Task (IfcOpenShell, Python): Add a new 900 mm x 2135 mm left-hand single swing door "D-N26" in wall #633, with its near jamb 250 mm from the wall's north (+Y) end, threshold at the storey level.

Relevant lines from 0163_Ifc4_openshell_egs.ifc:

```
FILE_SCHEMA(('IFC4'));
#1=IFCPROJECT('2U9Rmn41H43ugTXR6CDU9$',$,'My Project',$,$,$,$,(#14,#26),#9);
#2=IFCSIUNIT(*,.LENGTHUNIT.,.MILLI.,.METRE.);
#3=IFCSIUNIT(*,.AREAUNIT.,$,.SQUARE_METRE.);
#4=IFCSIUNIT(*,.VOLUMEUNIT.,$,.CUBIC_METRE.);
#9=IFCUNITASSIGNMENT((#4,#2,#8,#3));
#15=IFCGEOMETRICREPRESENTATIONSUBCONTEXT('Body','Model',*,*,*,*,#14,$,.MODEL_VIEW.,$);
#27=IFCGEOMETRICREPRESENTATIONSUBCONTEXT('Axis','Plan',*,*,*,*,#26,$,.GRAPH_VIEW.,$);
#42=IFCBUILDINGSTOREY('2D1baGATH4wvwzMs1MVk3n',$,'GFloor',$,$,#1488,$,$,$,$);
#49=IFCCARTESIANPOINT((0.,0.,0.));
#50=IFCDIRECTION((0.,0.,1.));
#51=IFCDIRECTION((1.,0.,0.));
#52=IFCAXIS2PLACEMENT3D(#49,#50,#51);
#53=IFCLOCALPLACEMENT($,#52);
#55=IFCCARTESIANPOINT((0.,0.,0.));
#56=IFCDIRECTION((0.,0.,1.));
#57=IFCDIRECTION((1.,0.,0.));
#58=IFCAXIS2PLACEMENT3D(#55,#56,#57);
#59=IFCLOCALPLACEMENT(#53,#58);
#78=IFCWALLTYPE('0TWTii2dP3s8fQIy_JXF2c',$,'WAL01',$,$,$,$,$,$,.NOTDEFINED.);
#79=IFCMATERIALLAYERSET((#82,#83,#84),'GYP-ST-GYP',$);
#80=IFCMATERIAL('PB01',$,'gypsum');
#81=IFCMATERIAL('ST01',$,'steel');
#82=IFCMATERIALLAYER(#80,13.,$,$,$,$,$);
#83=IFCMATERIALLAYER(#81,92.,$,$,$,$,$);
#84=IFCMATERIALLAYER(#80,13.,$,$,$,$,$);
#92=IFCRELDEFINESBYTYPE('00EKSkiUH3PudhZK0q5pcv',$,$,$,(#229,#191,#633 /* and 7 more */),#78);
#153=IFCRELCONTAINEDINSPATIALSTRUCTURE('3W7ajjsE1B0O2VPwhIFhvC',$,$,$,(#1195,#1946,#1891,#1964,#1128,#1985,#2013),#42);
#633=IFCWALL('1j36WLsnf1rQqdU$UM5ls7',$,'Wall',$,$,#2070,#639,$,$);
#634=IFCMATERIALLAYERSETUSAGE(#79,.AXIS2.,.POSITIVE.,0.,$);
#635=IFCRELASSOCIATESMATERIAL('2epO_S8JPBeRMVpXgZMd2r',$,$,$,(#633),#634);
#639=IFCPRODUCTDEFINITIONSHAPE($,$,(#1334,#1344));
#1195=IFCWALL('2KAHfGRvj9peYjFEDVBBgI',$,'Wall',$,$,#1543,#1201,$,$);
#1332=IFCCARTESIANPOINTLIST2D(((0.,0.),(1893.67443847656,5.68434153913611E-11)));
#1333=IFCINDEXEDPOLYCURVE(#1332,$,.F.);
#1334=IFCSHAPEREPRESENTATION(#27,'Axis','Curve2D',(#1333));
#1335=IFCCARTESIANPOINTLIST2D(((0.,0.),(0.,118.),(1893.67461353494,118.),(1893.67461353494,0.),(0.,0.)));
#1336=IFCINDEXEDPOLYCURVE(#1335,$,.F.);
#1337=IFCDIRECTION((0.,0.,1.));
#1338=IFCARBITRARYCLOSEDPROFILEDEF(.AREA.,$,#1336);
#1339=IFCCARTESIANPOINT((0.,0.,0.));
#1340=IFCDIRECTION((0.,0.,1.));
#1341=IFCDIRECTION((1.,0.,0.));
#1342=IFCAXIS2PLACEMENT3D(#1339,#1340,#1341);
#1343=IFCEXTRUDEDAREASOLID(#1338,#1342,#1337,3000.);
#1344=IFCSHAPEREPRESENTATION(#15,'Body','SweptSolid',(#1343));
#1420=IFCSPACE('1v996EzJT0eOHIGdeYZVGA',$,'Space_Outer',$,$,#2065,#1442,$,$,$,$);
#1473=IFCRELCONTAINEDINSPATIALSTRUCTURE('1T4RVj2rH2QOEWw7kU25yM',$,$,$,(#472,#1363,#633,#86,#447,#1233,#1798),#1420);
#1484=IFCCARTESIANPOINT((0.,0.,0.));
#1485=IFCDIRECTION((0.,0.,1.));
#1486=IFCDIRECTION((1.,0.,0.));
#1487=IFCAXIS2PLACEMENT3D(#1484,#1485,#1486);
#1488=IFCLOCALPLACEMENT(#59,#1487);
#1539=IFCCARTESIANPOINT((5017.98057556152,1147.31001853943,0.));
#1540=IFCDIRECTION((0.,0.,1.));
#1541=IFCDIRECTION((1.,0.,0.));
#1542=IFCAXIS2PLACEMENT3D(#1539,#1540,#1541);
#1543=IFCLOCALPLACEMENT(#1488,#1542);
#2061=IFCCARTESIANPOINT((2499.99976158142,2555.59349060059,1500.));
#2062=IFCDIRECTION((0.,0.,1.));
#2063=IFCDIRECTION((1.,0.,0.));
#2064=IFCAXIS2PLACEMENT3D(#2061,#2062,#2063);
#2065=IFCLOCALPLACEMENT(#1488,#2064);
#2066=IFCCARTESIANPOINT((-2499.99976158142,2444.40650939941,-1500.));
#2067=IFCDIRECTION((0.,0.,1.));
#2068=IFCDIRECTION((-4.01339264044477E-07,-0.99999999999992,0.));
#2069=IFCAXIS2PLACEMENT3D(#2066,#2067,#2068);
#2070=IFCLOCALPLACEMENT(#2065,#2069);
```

```python
import numpy as np
import ifcopenshell
import ifcopenshell.api.feature
import ifcopenshell.api.geometry
import ifcopenshell.api.root
import ifcopenshell.api.spatial
import ifcopenshell.geom
import ifcopenshell.util.element
import ifcopenshell.util.placement
import ifcopenshell.util.representation
import ifcopenshell.util.shape
import ifcopenshell.util.unit

model = ifcopenshell.open("0163_Ifc4_openshell_egs.ifc")
unit_scale = ifcopenshell.util.unit.calculate_unit_scale(model)
settings = ifcopenshell.geom.settings()


def volume(element):
    """Net volume in cubic metres, openings subtracted."""
    shape = ifcopenshell.geom.create_shape(settings, element)
    return ifcopenshell.util.shape.get_volume(shape.geometry)


wall = model.by_guid("1j36WLsnf1rQqdU$UM5ls7")
storey = ifcopenshell.util.element.get_container(wall, ifc_class="IfcBuildingStorey")
context = ifcopenshell.util.representation.get_context(model, "Model", "Body", "MODEL_VIEW")
before = volume(wall)

width, height, from_end, sill = 0.9, 2.135, 0.25, 0.0  # metres

# The wall runs along its own X axis, and the end named is its -X end.
wall_shape = ifcopenshell.geom.create_shape(settings, wall)
x, y, z = ifcopenshell.util.shape.get_vertices(wall_shape.geometry).T
start = x.min() + from_end
face, thickness = float(y.min()), float(y.max() - y.min())
wall_matrix = ifcopenshell.util.placement.get_local_placement(wall.ObjectPlacement)
level = ifcopenshell.util.placement.get_local_placement(storey.ObjectPlacement)[2, 3]


def in_wall(x, y):
    """Placement at x, y metres in the wall's axes, at sill height."""
    matrix = wall_matrix.copy()
    matrix[:, 3] = wall_matrix @ np.array([x / unit_scale, y / unit_scale, 0.0, 1.0])
    matrix[2, 3] = level + sill / unit_scale
    return matrix


# Opening: a box that overshoots both wall faces by 50 mm.
opening = ifcopenshell.api.root.create_entity(model, ifc_class="IfcOpeningElement", predefined_type="OPENING")
box = ifcopenshell.api.geometry.add_wall_representation(
    model, context=context, length=width, height=height, thickness=thickness + 0.1
)
ifcopenshell.api.geometry.assign_representation(model, product=opening, representation=box)
ifcopenshell.api.geometry.edit_object_placement(model, product=opening, matrix=in_wall(start, face - 0.05), is_si=False)
ifcopenshell.api.feature.add_feature(model, feature=opening, element=wall)

door = ifcopenshell.api.root.create_entity(model, ifc_class="IfcDoor", name="D-N26", predefined_type="DOOR")
door.OverallWidth, door.OverallHeight = width / unit_scale, height / unit_scale
door.OperationType = "SINGLE_SWING_LEFT"
body = ifcopenshell.api.geometry.add_door_representation(
    model,
    context=context,
    overall_width=door.OverallWidth,
    overall_height=door.OverallHeight,
    operation_type="SINGLE_SWING_LEFT",
    lining_properties={"LiningDepth": thickness / unit_scale, "ThresholdDepth": thickness / unit_scale},
)
ifcopenshell.api.geometry.assign_representation(model, product=door, representation=body)
ifcopenshell.api.spatial.assign_container(model, products=[door], relating_structure=storey)
ifcopenshell.api.feature.add_filling(model, opening=opening, element=door)

# The lining spans the wall, so the door starts at the wall face.
ifcopenshell.api.geometry.edit_object_placement(model, product=door, matrix=in_wall(start, face), is_si=False)

after = volume(wall)

print(f"wall volume {before:.3f} -> {after:.3f} m3")

model.write("0163_Ifc4_openshell_egs-out.ifc")
```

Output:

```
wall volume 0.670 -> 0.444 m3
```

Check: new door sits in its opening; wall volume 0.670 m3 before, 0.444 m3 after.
